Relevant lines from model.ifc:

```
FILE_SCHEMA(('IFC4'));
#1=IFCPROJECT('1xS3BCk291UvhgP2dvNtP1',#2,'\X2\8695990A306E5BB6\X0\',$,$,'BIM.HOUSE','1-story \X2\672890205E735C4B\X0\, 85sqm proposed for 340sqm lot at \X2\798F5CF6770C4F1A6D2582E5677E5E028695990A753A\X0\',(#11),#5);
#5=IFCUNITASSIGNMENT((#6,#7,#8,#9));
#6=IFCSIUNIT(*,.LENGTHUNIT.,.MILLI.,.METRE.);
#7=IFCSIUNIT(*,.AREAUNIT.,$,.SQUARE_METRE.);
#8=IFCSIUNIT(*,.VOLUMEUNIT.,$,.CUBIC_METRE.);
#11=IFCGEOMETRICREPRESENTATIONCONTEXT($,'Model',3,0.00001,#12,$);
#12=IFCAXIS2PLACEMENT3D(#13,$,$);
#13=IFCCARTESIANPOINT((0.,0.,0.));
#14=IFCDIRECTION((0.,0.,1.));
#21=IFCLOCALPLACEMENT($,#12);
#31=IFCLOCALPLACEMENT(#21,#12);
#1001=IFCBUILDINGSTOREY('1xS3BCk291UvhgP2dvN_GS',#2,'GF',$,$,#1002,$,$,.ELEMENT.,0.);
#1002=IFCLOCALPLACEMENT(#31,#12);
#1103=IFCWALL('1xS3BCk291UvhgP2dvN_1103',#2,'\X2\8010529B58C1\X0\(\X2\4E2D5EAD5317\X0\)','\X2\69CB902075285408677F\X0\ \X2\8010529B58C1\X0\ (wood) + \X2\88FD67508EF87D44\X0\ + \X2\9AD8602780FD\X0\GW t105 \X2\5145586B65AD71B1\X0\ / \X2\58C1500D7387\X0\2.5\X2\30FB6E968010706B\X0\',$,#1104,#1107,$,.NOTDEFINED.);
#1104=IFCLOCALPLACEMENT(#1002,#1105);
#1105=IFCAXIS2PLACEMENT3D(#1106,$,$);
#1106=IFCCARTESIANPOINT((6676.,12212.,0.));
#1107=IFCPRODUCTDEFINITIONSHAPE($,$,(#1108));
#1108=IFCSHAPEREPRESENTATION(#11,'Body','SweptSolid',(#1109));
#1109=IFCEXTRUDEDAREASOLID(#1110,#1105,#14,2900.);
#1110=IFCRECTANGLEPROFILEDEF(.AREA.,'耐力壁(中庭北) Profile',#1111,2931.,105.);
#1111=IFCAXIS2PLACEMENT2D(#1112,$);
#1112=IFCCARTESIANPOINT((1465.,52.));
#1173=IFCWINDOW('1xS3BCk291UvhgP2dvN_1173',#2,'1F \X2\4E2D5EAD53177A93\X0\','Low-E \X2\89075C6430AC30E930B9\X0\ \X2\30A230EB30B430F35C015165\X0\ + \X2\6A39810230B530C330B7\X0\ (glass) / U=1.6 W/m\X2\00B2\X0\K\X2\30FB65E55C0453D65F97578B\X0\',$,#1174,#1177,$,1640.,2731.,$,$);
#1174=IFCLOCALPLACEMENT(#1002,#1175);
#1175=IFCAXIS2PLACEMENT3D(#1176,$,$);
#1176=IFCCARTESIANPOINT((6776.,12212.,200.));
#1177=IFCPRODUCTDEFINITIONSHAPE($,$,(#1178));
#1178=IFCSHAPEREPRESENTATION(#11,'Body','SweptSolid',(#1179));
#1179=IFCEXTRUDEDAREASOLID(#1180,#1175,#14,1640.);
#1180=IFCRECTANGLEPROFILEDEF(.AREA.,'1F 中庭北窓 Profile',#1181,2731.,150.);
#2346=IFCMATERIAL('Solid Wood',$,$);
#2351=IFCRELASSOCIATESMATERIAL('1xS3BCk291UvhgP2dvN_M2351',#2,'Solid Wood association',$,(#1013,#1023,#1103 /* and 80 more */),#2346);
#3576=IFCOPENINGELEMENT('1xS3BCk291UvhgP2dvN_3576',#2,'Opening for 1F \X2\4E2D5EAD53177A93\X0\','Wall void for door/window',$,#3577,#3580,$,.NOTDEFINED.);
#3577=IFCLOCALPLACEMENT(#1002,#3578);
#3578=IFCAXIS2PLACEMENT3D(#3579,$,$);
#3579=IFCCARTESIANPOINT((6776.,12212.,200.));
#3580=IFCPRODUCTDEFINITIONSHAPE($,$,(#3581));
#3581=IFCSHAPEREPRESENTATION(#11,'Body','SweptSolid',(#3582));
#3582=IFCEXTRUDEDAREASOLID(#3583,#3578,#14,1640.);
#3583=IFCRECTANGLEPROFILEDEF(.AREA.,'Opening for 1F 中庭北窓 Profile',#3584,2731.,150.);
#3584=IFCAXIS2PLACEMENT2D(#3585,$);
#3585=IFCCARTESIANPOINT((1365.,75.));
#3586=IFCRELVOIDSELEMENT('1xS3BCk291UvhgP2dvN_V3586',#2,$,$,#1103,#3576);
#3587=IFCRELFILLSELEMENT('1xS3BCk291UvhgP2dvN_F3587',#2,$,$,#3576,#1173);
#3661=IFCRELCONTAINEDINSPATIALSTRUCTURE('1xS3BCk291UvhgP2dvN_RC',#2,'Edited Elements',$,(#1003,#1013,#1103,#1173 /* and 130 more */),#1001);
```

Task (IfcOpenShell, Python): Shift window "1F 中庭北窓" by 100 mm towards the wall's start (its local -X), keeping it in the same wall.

```python
import ifcopenshell
import ifcopenshell.api.geometry
import ifcopenshell.util.placement
import ifcopenshell.util.unit

model = ifcopenshell.open("model.ifc")
unit_scale = ifcopenshell.util.unit.calculate_unit_scale(model)

window = model.by_id(1173)
opening = window.FillsVoids[0].RelatingOpeningElement
wall = opening.VoidsElements[0].RelatingBuildingElement

wall_matrix = ifcopenshell.util.placement.get_local_placement(wall.ObjectPlacement)
shift = wall_matrix[:3, 0] * -0.1 / unit_scale
before = ifcopenshell.util.placement.get_local_placement(window.ObjectPlacement)[:3, 3].copy()

# The window is not placed relative to its opening, so move both.
for product in (opening, window):
    matrix = ifcopenshell.util.placement.get_local_placement(product.ObjectPlacement)
    matrix[:3, 3] += shift
    ifcopenshell.api.geometry.edit_object_placement(model, product=product, matrix=matrix, is_si=False)

after = ifcopenshell.util.placement.get_local_placement(window.ObjectPlacement)[:3, 3]
print("window moved by", (after - before).round(3) + 0.0)

model.write("model_v2.ifc")
```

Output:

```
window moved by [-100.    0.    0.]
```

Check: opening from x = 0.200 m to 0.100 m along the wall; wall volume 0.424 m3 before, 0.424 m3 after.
